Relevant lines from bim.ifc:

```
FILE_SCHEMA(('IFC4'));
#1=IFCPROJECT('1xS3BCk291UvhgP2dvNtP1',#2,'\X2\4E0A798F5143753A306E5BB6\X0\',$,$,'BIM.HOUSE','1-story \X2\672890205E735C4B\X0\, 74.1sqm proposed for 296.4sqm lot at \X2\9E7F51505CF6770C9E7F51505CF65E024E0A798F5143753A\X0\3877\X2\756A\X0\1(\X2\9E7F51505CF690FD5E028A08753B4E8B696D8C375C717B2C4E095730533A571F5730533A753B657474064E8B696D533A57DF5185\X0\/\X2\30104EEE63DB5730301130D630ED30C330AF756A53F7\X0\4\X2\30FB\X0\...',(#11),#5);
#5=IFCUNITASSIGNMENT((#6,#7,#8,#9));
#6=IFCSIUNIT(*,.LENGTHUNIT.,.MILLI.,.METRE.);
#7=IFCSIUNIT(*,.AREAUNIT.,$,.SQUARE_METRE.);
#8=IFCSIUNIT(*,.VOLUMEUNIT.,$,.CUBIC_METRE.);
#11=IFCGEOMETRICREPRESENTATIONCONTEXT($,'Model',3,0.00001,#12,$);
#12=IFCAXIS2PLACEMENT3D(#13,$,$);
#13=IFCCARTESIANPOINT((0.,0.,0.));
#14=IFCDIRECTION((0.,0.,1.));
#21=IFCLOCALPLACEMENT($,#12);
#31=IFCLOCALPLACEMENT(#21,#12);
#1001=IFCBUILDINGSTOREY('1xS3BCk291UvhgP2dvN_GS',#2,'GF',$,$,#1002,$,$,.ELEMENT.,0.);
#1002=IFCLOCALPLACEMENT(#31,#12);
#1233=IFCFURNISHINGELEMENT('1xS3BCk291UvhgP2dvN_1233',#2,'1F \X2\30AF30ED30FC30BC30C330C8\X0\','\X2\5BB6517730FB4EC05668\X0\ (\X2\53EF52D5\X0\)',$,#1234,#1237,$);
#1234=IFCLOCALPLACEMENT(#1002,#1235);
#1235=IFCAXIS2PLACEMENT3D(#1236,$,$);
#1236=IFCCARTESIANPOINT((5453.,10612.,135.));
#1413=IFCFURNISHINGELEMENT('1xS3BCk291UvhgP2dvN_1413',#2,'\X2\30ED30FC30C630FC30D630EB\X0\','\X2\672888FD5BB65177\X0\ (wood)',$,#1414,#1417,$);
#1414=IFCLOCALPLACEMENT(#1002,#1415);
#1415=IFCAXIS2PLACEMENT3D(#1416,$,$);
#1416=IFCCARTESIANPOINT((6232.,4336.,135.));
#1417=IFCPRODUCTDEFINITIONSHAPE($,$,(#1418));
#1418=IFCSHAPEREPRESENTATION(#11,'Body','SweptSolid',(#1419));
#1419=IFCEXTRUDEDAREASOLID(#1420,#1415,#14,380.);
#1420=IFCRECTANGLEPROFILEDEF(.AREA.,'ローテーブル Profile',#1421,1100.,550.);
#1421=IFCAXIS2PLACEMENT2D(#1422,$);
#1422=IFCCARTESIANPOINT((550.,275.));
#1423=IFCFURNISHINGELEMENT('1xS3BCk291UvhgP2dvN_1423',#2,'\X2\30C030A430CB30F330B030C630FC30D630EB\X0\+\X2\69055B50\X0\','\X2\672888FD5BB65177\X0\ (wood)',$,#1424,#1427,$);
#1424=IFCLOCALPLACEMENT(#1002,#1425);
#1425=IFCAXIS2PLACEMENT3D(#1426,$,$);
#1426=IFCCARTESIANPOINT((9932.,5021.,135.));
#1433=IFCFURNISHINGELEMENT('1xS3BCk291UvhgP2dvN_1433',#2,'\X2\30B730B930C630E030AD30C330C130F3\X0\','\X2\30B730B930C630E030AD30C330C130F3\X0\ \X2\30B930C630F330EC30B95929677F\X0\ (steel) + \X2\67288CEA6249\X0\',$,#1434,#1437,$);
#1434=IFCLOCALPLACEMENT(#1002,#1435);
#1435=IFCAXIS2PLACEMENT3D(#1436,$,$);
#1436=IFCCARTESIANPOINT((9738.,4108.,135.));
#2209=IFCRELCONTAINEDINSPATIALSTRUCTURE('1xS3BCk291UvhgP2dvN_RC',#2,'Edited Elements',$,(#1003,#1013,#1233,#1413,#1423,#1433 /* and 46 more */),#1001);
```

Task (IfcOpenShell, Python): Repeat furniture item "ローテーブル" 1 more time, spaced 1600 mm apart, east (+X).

```python
import numpy as np
import ifcopenshell
import ifcopenshell.api.geometry
import ifcopenshell.api.root
import ifcopenshell.util.element
import ifcopenshell.util.placement

model = ifcopenshell.open("bim.ifc")


def reuse_history(source, copy):
    """copy_class also copies each property set's owner history, people and application; keep the originals."""
    for rel in copy.IsDefinedBy:
        if rel.is_a("IfcRelDefinesByProperties") and (history := rel.RelatingPropertyDefinition.OwnerHistory):
            rel.RelatingPropertyDefinition.OwnerHistory = source.OwnerHistory
            ifcopenshell.util.element.remove_deep2(model, history)


source = model.by_id(1413)
base = ifcopenshell.util.placement.get_local_placement(source.ObjectPlacement)
step = np.array([1.0, 0.0, 0.0]) * 1600.0

for i in range(1, 2):
    copy = ifcopenshell.api.root.copy_class(model, product=source)
    copy.Representation = ifcopenshell.util.element.copy_deep(
        model, source.Representation, exclude=["IfcGeometricRepresentationContext", "IfcRepresentationMap"]
    )
    reuse_history(source, copy)
    matrix = base.copy()
    matrix[:3, 3] += i * step
    print("added at", matrix[:3, 3].round(3) + 0.0)
    ifcopenshell.api.geometry.edit_object_placement(model, product=copy, matrix=matrix, is_si=False)

model.write("bim_rev.ifc")
```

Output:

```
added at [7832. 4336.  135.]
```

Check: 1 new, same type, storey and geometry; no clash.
